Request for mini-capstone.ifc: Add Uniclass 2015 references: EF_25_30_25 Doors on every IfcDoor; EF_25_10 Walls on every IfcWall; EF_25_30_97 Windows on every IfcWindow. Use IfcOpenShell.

First a look at what the model holds.

```python
import ifcopenshell

model = ifcopenshell.open("mini-capstone.ifc")
print(model.schema)
print("classifications:", [c.Name for c in model.by_type("IfcClassification")])
for ifc_class in ("IfcDoor", "IfcRoof", "IfcStair", "IfcWall", "IfcWindow"):
    print(ifc_class, len(model.by_type(ifc_class)))
```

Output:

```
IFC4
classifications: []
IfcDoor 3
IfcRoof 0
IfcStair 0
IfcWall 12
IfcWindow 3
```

```python
import ifcopenshell
import ifcopenshell.api.classification

model = ifcopenshell.open("mini-capstone.ifc")

system = ifcopenshell.api.classification.add_classification(model, classification="Uniclass 2015")

codes = {
    "IfcDoor": ("EF_25_30_25", "Doors"),
    "IfcWall": ("EF_25_10", "Walls"),
    "IfcWindow": ("EF_25_30_97", "Windows"),
}
for ifc_class, (code, name) in codes.items():
    products = model.by_type(ifc_class)
    ifcopenshell.api.classification.add_reference(
        model, products=products, classification=system, identification=code, name=name
    )
    print(code, len(products))

model.write("mini-capstone_v2.ifc")
```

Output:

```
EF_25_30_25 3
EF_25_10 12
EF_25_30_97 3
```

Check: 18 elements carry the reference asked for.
